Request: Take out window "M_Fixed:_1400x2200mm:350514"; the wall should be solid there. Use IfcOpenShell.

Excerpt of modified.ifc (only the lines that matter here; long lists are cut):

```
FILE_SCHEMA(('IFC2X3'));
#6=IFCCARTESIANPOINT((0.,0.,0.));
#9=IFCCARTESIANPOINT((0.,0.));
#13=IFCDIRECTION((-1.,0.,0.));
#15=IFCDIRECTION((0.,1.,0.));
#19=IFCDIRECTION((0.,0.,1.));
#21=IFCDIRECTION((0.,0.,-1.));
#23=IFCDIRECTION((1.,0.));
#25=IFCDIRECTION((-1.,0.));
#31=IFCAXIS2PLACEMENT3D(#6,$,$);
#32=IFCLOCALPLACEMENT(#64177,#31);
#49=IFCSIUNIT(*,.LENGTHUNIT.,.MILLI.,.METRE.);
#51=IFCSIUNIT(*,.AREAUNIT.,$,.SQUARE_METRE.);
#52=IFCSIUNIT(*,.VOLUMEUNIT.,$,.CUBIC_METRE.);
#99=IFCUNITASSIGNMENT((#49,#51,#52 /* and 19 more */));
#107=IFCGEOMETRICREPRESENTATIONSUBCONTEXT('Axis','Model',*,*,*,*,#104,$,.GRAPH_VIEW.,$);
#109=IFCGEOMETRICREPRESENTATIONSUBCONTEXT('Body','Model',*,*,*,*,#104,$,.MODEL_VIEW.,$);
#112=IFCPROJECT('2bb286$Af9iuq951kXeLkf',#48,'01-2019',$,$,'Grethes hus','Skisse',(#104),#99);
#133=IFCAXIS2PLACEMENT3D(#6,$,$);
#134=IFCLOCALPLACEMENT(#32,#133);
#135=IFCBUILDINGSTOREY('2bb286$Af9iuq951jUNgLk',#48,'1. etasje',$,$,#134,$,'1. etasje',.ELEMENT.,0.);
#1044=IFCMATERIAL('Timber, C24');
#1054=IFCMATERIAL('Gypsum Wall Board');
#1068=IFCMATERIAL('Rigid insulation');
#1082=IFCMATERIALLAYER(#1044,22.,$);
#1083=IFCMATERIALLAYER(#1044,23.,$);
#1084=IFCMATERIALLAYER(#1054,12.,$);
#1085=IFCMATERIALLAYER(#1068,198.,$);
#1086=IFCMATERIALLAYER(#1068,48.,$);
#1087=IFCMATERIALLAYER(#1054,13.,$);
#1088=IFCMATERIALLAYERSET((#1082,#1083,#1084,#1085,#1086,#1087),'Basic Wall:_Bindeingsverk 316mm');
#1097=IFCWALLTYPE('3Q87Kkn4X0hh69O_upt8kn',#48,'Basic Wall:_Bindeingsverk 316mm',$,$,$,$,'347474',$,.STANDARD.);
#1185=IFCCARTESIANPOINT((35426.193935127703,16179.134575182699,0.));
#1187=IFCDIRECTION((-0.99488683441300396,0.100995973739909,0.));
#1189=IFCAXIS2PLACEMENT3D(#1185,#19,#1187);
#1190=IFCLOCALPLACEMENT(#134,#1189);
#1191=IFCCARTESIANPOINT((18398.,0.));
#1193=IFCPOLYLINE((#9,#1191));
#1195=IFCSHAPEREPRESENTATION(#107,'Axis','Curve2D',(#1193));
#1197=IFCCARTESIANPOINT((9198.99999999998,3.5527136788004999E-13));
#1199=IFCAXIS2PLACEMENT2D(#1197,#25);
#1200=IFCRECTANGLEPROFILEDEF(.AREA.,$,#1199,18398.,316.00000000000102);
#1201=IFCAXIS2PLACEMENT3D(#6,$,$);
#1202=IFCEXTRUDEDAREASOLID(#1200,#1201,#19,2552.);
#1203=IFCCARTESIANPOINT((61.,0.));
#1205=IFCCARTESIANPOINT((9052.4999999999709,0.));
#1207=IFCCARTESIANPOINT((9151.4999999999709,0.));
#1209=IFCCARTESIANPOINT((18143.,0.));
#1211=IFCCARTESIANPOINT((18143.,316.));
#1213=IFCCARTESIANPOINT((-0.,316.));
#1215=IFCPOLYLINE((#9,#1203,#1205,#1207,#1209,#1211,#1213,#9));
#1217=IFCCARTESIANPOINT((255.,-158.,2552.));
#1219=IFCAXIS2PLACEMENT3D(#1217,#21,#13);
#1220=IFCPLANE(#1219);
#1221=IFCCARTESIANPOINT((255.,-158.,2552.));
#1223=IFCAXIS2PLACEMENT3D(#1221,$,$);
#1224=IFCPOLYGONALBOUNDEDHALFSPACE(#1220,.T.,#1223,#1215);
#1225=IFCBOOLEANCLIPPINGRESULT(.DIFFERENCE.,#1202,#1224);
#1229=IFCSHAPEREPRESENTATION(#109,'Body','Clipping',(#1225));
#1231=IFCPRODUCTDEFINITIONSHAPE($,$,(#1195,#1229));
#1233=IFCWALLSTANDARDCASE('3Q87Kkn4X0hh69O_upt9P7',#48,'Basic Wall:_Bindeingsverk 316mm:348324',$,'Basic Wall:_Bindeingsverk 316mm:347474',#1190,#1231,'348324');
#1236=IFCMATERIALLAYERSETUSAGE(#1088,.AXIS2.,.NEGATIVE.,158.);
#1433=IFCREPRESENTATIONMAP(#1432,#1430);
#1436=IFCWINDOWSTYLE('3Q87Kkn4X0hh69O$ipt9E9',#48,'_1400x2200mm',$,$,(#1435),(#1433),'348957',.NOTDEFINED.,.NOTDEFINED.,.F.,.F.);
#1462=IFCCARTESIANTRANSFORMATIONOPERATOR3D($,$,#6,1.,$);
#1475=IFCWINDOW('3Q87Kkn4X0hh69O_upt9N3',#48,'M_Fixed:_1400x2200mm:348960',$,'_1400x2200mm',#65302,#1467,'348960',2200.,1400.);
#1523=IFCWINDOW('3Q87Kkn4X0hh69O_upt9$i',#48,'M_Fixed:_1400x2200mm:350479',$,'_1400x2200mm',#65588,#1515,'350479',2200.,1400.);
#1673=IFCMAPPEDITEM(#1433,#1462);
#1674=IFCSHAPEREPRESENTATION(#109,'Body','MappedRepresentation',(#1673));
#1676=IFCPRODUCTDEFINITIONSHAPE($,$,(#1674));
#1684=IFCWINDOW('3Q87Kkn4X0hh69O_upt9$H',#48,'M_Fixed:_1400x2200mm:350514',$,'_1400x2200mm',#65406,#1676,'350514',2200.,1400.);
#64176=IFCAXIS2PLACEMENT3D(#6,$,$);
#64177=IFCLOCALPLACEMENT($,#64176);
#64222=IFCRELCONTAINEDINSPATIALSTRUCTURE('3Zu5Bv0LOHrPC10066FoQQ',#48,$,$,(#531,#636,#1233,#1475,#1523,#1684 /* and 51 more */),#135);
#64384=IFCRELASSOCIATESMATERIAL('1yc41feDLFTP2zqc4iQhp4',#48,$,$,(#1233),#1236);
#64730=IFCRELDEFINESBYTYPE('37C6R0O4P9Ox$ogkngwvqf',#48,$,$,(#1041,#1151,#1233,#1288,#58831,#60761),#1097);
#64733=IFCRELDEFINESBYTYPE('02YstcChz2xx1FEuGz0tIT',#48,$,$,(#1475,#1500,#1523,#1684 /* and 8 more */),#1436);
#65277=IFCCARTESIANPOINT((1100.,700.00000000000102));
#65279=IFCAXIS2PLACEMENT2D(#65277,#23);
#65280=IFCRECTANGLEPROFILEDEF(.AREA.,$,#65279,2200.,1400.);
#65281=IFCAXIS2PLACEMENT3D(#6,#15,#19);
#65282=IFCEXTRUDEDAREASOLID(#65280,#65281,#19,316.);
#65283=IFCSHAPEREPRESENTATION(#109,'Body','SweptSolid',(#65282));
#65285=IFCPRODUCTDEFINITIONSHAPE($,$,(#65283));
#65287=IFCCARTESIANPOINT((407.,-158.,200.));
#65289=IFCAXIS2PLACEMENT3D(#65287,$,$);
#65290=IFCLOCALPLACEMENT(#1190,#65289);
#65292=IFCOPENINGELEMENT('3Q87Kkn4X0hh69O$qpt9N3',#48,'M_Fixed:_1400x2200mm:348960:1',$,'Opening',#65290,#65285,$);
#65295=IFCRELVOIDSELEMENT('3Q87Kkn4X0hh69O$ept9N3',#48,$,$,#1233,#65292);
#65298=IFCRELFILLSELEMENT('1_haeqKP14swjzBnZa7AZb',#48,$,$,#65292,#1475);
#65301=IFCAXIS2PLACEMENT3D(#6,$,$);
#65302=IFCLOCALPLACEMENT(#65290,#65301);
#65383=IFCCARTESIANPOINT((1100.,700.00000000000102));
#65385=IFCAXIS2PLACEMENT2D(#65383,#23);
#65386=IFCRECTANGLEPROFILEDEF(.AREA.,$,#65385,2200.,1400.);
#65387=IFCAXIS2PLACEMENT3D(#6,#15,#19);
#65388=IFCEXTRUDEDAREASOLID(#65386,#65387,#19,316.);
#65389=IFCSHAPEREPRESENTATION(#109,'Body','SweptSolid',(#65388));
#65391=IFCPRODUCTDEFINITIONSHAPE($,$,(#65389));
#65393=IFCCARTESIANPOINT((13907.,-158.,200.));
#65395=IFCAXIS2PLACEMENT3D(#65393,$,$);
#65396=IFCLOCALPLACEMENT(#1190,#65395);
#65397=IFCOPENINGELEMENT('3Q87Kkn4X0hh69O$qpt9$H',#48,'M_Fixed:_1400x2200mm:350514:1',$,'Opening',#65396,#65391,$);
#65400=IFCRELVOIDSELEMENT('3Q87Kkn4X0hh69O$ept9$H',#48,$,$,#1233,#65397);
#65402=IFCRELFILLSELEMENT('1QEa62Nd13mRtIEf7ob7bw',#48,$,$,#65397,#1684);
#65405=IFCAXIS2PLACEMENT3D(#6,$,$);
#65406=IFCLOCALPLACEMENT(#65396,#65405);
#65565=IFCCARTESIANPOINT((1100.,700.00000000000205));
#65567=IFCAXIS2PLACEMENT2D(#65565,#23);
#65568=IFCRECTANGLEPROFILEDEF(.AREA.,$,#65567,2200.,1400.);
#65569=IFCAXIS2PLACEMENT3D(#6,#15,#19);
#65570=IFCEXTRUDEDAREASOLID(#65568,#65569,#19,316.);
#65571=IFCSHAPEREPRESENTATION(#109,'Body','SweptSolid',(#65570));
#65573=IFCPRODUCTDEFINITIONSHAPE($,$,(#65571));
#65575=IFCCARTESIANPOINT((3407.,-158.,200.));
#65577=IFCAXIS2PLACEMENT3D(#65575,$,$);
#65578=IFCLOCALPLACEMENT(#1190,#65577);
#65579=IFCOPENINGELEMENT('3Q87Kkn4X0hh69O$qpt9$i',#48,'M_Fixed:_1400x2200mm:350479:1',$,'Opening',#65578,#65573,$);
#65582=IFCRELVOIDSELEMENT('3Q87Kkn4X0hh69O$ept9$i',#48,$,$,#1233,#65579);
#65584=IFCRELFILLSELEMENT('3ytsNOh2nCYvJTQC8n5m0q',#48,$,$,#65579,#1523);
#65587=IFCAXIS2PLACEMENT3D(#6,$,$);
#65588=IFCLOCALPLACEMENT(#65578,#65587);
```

```python
import ifcopenshell
import ifcopenshell.api.feature
import ifcopenshell.api.root
import ifcopenshell.geom
import ifcopenshell.util.shape

model = ifcopenshell.open("modified.ifc")
settings = ifcopenshell.geom.settings()


def volume(element):
    """Net volume in cubic metres, openings subtracted."""
    shape = ifcopenshell.geom.create_shape(settings, element)
    return ifcopenshell.util.shape.get_volume(shape.geometry)


window = model.by_guid("3Q87Kkn4X0hh69O_upt9$H")
opening = window.FillsVoids[0].RelatingOpeningElement
wall = opening.VoidsElements[0].RelatingBuildingElement
before = volume(wall)

ifcopenshell.api.root.remove_product(model, product=window)
ifcopenshell.api.feature.remove_feature(model, feature=opening)

after = volume(wall)

print(f"wall volume {before:.3f} -> {after:.3f} m3")

model.write("modified_updated.ifc")
```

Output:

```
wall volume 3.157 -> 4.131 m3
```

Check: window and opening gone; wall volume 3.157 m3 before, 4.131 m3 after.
